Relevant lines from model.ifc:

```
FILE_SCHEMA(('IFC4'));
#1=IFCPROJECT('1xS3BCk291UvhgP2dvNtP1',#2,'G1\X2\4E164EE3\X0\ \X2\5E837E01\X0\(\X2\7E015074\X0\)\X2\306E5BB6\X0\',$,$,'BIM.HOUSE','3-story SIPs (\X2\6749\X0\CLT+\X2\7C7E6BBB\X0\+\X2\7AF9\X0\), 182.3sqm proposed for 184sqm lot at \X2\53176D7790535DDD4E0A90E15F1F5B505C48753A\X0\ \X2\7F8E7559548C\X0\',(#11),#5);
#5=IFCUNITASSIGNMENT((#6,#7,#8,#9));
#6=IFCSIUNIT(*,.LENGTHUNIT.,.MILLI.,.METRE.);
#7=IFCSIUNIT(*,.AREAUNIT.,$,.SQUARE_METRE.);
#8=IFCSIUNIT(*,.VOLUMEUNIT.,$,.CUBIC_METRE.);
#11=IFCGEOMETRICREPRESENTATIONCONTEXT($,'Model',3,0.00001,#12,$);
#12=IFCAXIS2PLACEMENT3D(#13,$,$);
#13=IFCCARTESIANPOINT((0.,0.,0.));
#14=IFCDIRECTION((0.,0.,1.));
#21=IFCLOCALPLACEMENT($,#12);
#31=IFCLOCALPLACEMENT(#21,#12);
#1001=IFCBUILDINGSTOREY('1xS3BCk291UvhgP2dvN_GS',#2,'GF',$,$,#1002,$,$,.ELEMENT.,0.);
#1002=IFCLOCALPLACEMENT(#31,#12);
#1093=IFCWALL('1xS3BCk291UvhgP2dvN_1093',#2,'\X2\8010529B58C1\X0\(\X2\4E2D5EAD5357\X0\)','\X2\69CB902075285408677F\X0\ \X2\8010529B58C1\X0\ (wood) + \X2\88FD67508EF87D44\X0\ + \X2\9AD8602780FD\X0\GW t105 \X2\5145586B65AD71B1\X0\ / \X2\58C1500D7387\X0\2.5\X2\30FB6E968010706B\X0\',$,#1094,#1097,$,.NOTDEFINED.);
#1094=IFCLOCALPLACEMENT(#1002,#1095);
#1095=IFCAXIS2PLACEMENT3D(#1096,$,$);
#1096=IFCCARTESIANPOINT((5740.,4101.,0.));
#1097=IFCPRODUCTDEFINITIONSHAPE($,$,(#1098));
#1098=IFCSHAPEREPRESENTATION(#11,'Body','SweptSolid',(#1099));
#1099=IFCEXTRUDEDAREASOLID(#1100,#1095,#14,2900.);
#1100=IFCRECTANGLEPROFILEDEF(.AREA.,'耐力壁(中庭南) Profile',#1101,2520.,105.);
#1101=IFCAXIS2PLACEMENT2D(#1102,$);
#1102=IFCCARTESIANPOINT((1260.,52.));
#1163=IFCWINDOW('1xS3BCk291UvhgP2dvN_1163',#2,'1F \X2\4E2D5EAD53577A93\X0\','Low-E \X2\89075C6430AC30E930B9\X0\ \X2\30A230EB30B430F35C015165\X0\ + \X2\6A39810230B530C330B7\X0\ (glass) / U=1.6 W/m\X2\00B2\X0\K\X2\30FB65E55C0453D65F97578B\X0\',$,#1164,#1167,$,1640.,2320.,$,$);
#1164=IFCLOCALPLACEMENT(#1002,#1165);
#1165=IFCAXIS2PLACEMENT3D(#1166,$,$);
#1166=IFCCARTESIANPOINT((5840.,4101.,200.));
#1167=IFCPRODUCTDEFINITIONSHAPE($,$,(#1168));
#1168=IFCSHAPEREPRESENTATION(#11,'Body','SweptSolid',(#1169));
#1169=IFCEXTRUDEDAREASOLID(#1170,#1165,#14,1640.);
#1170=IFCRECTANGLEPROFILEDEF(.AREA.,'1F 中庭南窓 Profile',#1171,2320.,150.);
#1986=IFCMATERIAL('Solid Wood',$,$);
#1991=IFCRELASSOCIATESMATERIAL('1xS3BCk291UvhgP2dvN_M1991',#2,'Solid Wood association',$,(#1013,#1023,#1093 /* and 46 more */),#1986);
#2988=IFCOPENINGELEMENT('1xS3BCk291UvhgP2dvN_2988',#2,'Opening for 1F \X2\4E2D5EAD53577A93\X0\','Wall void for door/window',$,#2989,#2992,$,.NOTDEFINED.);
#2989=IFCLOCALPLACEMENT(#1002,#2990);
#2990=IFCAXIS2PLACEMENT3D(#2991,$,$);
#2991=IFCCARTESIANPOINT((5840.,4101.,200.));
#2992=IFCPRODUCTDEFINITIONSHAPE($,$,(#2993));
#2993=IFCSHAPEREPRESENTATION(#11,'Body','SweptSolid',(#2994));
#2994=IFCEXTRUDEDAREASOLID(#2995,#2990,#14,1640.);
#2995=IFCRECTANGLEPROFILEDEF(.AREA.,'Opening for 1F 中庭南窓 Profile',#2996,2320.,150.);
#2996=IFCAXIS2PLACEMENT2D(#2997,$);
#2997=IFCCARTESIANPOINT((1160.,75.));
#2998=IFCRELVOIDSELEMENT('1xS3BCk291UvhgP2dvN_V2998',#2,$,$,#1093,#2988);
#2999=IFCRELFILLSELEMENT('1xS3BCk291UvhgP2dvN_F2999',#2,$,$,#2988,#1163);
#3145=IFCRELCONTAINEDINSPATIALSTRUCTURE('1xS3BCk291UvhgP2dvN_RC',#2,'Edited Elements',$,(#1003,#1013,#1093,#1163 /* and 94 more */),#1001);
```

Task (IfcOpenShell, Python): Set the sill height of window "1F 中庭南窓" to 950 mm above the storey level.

```python
import numpy as np
import ifcopenshell
import ifcopenshell.api.geometry
import ifcopenshell.geom
import ifcopenshell.util.element
import ifcopenshell.util.placement
import ifcopenshell.util.shape
import ifcopenshell.util.unit

model = ifcopenshell.open("model.ifc")
unit_scale = ifcopenshell.util.unit.calculate_unit_scale(model)

window = model.by_guid("1xS3BCk291UvhgP2dvN_1163")
opening = window.FillsVoids[0].RelatingOpeningElement
storey = ifcopenshell.util.element.get_container(window, ifc_class="IfcBuildingStorey")
level = ifcopenshell.util.placement.get_local_placement(storey.ObjectPlacement)[2, 3]

# The opening's origin need not be at the sill, so measure its lowest point.
shape = ifcopenshell.geom.create_shape(ifcopenshell.geom.settings(), opening)
bottom = ifcopenshell.util.shape.get_shape_bottom_elevation(shape, shape.geometry) / unit_scale
dz = level + 950.0 - bottom

shift = np.array([0.0, 0.0, dz])
# The window is not placed relative to its opening, so move both.
for product in (opening, window):
    matrix = ifcopenshell.util.placement.get_local_placement(product.ObjectPlacement)
    matrix[:3, 3] += shift
    ifcopenshell.api.geometry.edit_object_placement(model, product=product, matrix=matrix, is_si=False)

print(f"moved by {dz * unit_scale:+.3f} m")

model.write("model_updated.ifc")
```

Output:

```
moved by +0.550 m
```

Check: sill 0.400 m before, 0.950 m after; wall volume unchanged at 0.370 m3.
